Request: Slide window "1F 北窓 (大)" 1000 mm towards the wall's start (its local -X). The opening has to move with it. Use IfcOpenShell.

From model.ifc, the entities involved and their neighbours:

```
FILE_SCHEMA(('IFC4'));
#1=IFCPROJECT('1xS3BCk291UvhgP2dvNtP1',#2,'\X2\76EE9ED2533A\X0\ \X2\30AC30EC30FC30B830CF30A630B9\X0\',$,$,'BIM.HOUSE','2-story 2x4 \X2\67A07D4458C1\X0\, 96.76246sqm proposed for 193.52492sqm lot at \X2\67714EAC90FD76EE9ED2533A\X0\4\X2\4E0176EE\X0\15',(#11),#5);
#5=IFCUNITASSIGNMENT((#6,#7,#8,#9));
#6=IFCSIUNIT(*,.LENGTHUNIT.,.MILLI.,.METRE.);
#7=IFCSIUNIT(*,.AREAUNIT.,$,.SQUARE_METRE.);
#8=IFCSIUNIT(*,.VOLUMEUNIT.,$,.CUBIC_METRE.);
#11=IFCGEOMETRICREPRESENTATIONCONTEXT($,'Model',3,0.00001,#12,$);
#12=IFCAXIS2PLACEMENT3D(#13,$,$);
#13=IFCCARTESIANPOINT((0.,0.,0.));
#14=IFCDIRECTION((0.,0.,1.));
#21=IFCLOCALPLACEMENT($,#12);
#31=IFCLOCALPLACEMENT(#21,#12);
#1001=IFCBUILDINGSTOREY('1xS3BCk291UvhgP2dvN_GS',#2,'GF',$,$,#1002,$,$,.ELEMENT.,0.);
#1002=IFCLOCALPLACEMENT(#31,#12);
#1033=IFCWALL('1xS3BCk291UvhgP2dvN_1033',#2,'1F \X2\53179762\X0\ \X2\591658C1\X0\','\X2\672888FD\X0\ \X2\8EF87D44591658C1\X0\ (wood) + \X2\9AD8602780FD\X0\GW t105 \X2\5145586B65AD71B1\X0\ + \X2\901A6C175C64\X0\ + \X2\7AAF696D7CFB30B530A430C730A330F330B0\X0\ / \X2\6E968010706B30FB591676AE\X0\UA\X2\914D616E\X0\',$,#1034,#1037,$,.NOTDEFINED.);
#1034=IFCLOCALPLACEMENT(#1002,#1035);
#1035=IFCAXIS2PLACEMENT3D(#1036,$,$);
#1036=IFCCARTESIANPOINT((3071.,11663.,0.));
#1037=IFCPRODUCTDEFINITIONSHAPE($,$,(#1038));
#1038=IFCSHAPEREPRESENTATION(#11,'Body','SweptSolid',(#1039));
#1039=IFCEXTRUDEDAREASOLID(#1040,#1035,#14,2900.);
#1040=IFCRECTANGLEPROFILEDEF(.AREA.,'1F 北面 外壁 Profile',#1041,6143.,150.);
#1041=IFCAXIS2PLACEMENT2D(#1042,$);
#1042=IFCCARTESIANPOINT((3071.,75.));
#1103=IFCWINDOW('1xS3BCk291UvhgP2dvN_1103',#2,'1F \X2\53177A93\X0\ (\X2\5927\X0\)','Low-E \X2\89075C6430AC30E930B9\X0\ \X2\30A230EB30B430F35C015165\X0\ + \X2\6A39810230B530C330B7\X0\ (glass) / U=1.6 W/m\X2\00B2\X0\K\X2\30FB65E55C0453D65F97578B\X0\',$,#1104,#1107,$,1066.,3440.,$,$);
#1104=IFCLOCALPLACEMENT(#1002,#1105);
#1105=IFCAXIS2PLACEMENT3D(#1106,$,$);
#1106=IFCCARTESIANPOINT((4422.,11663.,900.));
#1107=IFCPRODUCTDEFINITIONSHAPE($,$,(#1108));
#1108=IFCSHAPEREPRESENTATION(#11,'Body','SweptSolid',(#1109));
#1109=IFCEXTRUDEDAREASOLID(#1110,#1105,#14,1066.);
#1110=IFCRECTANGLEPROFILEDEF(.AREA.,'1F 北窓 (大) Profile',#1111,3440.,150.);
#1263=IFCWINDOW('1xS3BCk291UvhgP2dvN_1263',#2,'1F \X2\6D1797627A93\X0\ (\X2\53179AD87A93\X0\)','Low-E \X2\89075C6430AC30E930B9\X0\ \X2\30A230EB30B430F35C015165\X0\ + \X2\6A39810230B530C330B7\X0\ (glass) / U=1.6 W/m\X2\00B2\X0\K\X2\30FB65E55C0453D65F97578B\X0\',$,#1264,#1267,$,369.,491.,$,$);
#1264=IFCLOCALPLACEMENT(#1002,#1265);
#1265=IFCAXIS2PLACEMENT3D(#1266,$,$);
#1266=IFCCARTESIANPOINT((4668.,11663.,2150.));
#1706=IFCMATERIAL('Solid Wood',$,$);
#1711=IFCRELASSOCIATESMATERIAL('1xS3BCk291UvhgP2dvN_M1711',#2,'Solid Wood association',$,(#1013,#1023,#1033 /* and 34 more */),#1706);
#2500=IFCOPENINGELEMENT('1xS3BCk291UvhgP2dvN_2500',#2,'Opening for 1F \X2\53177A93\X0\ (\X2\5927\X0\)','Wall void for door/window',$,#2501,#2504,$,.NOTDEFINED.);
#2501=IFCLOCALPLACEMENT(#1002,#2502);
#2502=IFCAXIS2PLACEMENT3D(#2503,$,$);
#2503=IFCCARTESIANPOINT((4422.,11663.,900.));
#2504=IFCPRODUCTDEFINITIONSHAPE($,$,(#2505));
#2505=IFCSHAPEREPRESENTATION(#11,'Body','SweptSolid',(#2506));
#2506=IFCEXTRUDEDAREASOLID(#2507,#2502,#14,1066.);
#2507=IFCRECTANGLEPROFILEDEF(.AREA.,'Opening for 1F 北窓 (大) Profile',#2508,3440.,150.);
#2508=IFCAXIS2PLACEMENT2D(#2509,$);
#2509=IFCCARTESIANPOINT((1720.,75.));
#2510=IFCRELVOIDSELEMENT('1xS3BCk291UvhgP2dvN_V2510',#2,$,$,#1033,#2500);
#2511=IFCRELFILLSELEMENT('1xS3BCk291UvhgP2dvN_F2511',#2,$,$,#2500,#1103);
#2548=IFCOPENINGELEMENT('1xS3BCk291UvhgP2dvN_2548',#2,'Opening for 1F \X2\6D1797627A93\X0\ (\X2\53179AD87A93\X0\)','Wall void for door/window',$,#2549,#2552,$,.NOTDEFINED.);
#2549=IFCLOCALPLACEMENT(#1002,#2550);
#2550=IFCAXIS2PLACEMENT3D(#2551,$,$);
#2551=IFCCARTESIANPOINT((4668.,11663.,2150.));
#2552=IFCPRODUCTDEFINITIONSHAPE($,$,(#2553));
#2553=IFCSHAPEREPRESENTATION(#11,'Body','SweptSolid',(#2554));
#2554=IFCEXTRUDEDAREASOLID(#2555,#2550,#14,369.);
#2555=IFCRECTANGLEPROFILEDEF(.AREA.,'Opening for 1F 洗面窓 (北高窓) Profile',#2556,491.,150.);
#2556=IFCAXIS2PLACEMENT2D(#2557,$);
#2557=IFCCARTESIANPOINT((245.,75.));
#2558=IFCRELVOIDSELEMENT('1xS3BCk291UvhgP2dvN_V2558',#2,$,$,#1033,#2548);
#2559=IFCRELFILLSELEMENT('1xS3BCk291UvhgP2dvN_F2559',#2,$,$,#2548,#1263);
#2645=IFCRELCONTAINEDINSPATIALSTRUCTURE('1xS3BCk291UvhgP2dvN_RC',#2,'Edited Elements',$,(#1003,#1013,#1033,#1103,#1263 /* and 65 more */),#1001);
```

```python
import ifcopenshell
import ifcopenshell.api.geometry
import ifcopenshell.util.placement
import ifcopenshell.util.unit

model = ifcopenshell.open("model.ifc")
unit_scale = ifcopenshell.util.unit.calculate_unit_scale(model)

window = model.by_guid("1xS3BCk291UvhgP2dvN_1103")
opening = window.FillsVoids[0].RelatingOpeningElement
wall = opening.VoidsElements[0].RelatingBuildingElement

wall_matrix = ifcopenshell.util.placement.get_local_placement(wall.ObjectPlacement)
shift = wall_matrix[:3, 0] * -1 / unit_scale
before = ifcopenshell.util.placement.get_local_placement(window.ObjectPlacement)[:3, 3].copy()

# The window is not placed relative to its opening, so move both.
for product in (opening, window):
    matrix = ifcopenshell.util.placement.get_local_placement(product.ObjectPlacement)
    matrix[:3, 3] += shift
    ifcopenshell.api.geometry.edit_object_placement(model, product=product, matrix=matrix, is_si=False)

after = ifcopenshell.util.placement.get_local_placement(window.ObjectPlacement)[:3, 3]
print("window moved by", (after - before).round(3) + 0.0)

model.write("model_rev.ifc")
```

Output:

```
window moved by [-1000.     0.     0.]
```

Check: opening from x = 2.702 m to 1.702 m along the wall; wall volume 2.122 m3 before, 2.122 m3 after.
